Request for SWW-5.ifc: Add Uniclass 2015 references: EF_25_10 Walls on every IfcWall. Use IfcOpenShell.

First a look at what the model holds.

```python
import ifcopenshell

model = ifcopenshell.open("SWW-5.ifc")
print(model.schema)
print("classifications:", [c.Name for c in model.by_type("IfcClassification")])
for ifc_class in ("IfcDoor", "IfcRoof", "IfcStair", "IfcWall", "IfcWindow"):
    print(ifc_class, len(model.by_type(ifc_class)))
```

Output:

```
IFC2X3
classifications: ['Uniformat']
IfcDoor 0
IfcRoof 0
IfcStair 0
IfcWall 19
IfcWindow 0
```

```python
import ifcopenshell
import ifcopenshell.api.classification

model = ifcopenshell.open("SWW-5.ifc")

# IFC2X3 requires Source and Edition and has no link from the project to the system.
system = model.create_entity("IfcClassification", Source="NBS", Edition="2015", Name="Uniclass 2015")

codes = {
    "IfcWall": ("EF_25_10", "Walls"),
}
for ifc_class, (code, name) in codes.items():
    products = model.by_type(ifc_class)
    ifcopenshell.api.classification.add_reference(
        model, products=products, classification=system, identification=code, name=name
    )
    print(code, len(products))

model.write("SWW-5_edited.ifc")
```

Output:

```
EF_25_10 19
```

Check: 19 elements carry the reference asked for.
